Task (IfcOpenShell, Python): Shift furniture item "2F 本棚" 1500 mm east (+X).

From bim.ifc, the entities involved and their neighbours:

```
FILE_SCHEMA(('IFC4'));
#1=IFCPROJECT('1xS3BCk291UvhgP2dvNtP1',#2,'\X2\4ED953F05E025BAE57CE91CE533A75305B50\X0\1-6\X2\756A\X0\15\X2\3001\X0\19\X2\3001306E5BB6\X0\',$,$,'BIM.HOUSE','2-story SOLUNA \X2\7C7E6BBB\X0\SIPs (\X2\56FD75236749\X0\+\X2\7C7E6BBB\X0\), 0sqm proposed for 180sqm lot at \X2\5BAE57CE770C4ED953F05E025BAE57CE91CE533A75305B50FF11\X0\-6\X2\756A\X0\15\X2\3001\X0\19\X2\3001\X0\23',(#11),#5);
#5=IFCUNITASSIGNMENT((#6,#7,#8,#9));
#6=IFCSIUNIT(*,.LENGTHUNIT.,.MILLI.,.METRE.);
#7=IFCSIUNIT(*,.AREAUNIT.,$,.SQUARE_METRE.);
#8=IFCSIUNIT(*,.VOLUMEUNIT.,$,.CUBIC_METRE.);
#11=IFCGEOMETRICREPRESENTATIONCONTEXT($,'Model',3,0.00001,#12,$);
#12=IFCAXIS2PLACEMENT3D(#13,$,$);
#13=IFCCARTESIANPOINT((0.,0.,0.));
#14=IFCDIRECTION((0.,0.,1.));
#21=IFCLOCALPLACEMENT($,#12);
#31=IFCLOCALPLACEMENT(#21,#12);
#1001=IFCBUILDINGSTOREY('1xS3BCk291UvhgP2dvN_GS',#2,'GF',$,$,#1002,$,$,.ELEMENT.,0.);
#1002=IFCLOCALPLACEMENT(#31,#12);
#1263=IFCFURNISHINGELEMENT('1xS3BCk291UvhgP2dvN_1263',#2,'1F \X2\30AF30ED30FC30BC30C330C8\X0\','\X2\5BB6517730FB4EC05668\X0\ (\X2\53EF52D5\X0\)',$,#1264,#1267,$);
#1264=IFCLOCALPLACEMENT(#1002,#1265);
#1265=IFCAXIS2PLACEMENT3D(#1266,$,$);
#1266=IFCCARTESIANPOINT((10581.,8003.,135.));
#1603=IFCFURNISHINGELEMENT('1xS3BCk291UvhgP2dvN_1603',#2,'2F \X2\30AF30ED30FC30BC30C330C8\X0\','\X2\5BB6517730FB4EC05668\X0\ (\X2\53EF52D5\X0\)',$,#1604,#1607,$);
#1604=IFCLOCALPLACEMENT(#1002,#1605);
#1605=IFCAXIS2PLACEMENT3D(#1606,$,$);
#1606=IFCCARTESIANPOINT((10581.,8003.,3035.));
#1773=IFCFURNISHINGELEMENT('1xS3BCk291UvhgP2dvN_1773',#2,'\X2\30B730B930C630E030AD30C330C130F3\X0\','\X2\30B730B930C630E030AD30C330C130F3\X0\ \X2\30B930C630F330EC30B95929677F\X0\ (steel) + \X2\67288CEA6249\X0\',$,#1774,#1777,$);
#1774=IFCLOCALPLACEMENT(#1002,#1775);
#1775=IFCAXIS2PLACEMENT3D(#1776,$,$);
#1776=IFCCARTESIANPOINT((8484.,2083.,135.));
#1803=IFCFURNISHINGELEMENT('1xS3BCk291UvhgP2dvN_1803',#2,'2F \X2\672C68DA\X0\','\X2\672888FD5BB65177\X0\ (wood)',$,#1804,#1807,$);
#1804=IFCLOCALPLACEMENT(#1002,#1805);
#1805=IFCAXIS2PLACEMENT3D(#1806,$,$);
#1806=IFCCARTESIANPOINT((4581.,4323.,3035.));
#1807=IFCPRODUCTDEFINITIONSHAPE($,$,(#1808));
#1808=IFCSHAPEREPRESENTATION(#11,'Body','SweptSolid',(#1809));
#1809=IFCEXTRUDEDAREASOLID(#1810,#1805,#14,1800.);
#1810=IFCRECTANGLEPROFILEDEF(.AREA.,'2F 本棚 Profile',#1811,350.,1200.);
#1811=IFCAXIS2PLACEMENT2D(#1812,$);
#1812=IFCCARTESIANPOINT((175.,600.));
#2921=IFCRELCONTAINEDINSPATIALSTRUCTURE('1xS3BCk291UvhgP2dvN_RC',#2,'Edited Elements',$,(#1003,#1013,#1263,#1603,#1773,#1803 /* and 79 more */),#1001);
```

```python
import ifcopenshell
import ifcopenshell.api.geometry
import ifcopenshell.util.placement
import ifcopenshell.util.unit

model = ifcopenshell.open("bim.ifc")
unit_scale = ifcopenshell.util.unit.calculate_unit_scale(model)

item = model.by_guid("1xS3BCk291UvhgP2dvN_1803")
matrix = ifcopenshell.util.placement.get_local_placement(item.ObjectPlacement)
matrix[0, 3] += 1.5 / unit_scale
ifcopenshell.api.geometry.edit_object_placement(model, product=item, matrix=matrix, is_si=False)

print(ifcopenshell.util.placement.get_local_placement(item.ObjectPlacement).round(3) + 0.0)

model.write("bim_v2.ifc")
```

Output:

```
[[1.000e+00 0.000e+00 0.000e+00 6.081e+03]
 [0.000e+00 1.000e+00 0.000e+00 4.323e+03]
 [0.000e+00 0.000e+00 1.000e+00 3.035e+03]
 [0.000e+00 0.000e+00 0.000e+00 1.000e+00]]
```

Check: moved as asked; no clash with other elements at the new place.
